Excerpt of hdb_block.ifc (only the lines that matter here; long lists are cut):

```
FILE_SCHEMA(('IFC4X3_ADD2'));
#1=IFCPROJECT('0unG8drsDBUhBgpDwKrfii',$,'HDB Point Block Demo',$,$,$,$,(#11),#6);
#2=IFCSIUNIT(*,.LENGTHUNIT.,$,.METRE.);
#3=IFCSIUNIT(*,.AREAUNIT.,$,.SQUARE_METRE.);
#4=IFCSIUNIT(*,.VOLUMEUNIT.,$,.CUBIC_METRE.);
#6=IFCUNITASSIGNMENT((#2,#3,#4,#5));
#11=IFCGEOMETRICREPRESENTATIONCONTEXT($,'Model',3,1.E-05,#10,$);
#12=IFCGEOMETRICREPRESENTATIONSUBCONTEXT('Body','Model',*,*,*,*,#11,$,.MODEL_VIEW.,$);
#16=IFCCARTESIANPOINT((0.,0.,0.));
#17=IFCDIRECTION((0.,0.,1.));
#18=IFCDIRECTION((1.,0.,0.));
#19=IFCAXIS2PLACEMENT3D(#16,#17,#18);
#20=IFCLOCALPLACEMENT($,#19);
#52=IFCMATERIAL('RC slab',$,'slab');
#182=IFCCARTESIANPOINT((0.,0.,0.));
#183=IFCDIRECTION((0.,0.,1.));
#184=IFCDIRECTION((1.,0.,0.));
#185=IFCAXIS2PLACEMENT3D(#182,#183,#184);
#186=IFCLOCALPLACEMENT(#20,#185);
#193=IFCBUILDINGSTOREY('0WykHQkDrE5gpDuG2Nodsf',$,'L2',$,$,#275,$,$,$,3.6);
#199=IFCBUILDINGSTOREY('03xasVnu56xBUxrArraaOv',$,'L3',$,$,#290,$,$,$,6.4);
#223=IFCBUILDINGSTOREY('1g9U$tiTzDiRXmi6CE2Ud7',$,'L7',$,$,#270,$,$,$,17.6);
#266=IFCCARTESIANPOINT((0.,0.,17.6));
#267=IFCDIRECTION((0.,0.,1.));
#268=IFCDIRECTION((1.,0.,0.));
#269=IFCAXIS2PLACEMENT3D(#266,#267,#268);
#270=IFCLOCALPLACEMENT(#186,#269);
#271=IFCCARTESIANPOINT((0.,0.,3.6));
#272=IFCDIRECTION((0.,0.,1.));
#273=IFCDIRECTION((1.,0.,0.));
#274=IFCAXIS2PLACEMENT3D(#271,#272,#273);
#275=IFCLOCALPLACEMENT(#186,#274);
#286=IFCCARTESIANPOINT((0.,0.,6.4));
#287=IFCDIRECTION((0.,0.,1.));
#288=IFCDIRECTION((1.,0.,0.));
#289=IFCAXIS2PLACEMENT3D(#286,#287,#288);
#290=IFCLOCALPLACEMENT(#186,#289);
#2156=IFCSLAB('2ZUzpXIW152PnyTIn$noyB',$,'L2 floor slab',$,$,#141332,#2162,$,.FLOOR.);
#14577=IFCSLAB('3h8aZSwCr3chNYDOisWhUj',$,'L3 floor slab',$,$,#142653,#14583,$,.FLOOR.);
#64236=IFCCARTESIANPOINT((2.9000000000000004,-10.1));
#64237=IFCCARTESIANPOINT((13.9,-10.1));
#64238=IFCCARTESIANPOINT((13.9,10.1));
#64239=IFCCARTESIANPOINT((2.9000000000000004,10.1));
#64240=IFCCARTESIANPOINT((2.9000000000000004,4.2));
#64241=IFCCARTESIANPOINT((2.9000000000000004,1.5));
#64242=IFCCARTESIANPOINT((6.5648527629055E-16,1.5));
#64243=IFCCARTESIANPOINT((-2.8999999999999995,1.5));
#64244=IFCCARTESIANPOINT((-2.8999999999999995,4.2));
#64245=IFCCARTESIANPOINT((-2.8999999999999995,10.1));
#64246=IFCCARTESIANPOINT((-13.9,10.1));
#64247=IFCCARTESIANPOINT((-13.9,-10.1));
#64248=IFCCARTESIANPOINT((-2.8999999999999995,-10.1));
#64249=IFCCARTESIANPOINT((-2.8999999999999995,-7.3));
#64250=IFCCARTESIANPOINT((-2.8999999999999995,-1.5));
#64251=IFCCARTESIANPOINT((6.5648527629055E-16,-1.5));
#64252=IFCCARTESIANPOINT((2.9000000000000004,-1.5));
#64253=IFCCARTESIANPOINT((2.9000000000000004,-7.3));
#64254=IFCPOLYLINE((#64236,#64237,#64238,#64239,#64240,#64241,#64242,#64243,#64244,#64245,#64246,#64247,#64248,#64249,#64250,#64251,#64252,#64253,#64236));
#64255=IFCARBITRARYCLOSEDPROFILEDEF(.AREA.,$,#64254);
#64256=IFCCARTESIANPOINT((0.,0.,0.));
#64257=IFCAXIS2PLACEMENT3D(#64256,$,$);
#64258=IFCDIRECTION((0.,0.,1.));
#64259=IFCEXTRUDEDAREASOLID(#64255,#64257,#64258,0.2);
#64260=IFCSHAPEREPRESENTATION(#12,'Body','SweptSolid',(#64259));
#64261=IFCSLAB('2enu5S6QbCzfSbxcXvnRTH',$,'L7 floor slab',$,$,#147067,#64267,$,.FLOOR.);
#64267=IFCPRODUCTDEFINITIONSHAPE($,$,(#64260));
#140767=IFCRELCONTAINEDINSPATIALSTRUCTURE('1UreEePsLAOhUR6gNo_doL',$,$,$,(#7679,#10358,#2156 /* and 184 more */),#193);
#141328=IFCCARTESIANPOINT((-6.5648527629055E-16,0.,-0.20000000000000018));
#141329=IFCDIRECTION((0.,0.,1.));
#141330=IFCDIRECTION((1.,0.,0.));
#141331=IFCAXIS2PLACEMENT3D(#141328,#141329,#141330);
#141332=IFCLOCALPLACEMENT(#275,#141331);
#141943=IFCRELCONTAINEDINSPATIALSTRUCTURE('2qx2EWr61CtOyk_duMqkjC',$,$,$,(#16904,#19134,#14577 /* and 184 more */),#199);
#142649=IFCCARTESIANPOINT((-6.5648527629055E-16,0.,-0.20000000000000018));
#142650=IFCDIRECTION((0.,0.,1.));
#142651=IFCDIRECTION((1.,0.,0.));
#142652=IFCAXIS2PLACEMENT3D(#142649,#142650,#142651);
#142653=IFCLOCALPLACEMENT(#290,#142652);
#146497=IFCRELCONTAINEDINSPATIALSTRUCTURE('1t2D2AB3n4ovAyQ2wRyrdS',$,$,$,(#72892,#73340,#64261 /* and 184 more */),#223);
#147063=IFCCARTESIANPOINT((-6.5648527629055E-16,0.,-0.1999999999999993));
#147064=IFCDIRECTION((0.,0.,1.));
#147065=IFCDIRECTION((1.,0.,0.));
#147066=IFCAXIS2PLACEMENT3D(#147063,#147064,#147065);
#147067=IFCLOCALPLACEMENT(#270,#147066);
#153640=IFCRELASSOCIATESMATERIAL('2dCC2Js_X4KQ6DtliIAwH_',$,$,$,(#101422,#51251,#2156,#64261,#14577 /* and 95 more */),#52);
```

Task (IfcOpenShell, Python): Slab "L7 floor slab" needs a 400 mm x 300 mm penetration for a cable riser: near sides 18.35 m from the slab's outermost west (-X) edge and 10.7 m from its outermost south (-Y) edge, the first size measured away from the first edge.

```python
import numpy as np
import ifcopenshell
import ifcopenshell.api.feature
import ifcopenshell.api.geometry
import ifcopenshell.api.root
import ifcopenshell.geom
import ifcopenshell.util.placement
import ifcopenshell.util.representation
import ifcopenshell.util.shape
import ifcopenshell.util.unit

model = ifcopenshell.open("hdb_block.ifc")
unit_scale = ifcopenshell.util.unit.calculate_unit_scale(model)
settings = ifcopenshell.geom.settings()


def volume(element):
    """Net volume in cubic metres, openings subtracted."""
    shape = ifcopenshell.geom.create_shape(settings, element)
    return ifcopenshell.util.shape.get_volume(shape.geometry)


slab = model.by_id(64261)
before = volume(slab)

# Extent in the slab's own axes, in metres. The edges named are its -X and -Y sides.
slab_shape = ifcopenshell.geom.create_shape(settings, slab)
vertices = ifcopenshell.util.shape.get_vertices(slab_shape.geometry)
x_min, y_min, bottom = vertices.min(axis=0)
top = vertices[:, 2].max()

opening = ifcopenshell.api.root.create_entity(model, ifc_class="IfcOpeningElement", name="Cable riser opening", predefined_type="OPENING")
context = ifcopenshell.util.representation.get_context(model, "Model", "Body", "MODEL_VIEW")
width, depth = 0.4, 0.3
outline = [(0.0, 0.0), (width, 0.0), (width, depth), (0.0, depth), (0.0, 0.0)]
# Overshoot both faces by 50 mm so the cut is clean.
shape = ifcopenshell.api.geometry.add_slab_representation(
    model, context=context, depth=top - bottom + 0.1, polyline=outline
)
ifcopenshell.api.geometry.assign_representation(model, product=opening, representation=shape)

matrix = ifcopenshell.util.placement.get_local_placement(slab.ObjectPlacement)
matrix[:, 3] = matrix @ np.append(np.array([x_min + 18.35, y_min + 10.7, bottom - 0.05]) / unit_scale, 1.0)
ifcopenshell.api.geometry.edit_object_placement(model, product=opening, matrix=matrix, is_si=False)
ifcopenshell.api.feature.add_feature(model, feature=opening, element=slab)

after = volume(slab)

print(f"slab volume {before:.3f} -> {after:.3f} m3")

model.write("hdb_block_v2.ifc")
```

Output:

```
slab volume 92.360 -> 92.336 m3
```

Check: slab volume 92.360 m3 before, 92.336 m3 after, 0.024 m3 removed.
